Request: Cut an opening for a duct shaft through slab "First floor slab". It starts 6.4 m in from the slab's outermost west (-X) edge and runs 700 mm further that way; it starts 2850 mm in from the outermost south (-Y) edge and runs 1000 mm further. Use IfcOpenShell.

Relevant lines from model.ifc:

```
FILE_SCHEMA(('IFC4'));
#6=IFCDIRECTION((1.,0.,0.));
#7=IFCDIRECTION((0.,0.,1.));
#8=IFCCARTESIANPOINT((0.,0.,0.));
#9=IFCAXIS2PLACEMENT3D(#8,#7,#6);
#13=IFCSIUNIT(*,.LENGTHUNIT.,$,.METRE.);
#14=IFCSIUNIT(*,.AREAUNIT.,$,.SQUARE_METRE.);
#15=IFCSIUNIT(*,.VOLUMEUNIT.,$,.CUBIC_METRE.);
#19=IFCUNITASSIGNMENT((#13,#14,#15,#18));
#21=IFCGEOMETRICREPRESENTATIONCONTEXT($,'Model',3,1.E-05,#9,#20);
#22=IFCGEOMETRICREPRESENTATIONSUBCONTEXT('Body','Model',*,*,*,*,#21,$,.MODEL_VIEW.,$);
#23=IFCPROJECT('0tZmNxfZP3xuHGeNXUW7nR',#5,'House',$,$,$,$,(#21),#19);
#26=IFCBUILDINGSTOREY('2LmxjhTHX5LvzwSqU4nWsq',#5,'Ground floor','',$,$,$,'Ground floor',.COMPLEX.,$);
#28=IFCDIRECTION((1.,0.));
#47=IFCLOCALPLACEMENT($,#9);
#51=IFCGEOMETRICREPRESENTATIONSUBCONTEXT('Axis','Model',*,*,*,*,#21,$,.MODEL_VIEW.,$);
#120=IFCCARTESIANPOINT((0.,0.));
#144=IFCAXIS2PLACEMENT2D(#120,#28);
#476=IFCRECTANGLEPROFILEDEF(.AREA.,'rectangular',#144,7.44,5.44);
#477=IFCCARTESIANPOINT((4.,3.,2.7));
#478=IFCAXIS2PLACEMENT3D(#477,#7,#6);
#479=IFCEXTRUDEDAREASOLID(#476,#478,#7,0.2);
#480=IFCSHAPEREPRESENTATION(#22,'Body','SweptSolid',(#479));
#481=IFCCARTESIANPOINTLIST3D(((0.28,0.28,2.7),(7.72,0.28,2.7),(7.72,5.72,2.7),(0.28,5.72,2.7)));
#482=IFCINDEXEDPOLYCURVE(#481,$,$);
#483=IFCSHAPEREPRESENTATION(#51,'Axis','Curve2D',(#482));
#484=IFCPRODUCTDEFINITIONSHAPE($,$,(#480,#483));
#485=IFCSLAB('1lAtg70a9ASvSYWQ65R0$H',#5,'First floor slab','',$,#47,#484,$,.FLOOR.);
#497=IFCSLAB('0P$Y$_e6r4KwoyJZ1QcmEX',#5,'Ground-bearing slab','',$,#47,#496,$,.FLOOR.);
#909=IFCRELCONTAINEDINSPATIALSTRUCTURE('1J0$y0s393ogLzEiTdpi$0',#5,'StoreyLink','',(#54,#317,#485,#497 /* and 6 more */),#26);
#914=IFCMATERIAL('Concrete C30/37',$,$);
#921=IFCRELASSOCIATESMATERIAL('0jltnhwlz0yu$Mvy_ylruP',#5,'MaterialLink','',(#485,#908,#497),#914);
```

```python
import numpy as np
import ifcopenshell
import ifcopenshell.api.feature
import ifcopenshell.api.geometry
import ifcopenshell.api.root
import ifcopenshell.geom
import ifcopenshell.util.placement
import ifcopenshell.util.representation
import ifcopenshell.util.shape
import ifcopenshell.util.unit

model = ifcopenshell.open("model.ifc")
unit_scale = ifcopenshell.util.unit.calculate_unit_scale(model)
settings = ifcopenshell.geom.settings()


def volume(element):
    """Net volume in cubic metres, openings subtracted."""
    shape = ifcopenshell.geom.create_shape(settings, element)
    return ifcopenshell.util.shape.get_volume(shape.geometry)


slab = model.by_guid("1lAtg70a9ASvSYWQ65R0$H")
before = volume(slab)

# Extent in the slab's own axes, in metres. The edges named are its -X and -Y sides.
slab_shape = ifcopenshell.geom.create_shape(settings, slab)
vertices = ifcopenshell.util.shape.get_vertices(slab_shape.geometry)
x_min, y_min, bottom = vertices.min(axis=0)
top = vertices[:, 2].max()

opening = ifcopenshell.api.root.create_entity(model, ifc_class="IfcOpeningElement", name="Duct shaft opening", predefined_type="OPENING")
context = ifcopenshell.util.representation.get_context(model, "Model", "Body", "MODEL_VIEW")
width, depth = 0.7, 1
outline = [(0.0, 0.0), (width, 0.0), (width, depth), (0.0, depth), (0.0, 0.0)]
# Overshoot both faces by 50 mm so the cut is clean.
shape = ifcopenshell.api.geometry.add_slab_representation(
    model, context=context, depth=top - bottom + 0.1, polyline=outline
)
ifcopenshell.api.geometry.assign_representation(model, product=opening, representation=shape)

matrix = ifcopenshell.util.placement.get_local_placement(slab.ObjectPlacement)
matrix[:, 3] = matrix @ np.append(np.array([x_min + 6.4, y_min + 2.85, bottom - 0.05]) / unit_scale, 1.0)
ifcopenshell.api.geometry.edit_object_placement(model, product=opening, matrix=matrix, is_si=False)
ifcopenshell.api.feature.add_feature(model, feature=opening, element=slab)

after = volume(slab)

print(f"slab volume {before:.3f} -> {after:.3f} m3")

model.write("model_updated.ifc")
```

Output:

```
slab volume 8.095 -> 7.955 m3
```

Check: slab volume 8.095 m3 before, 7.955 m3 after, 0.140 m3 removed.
